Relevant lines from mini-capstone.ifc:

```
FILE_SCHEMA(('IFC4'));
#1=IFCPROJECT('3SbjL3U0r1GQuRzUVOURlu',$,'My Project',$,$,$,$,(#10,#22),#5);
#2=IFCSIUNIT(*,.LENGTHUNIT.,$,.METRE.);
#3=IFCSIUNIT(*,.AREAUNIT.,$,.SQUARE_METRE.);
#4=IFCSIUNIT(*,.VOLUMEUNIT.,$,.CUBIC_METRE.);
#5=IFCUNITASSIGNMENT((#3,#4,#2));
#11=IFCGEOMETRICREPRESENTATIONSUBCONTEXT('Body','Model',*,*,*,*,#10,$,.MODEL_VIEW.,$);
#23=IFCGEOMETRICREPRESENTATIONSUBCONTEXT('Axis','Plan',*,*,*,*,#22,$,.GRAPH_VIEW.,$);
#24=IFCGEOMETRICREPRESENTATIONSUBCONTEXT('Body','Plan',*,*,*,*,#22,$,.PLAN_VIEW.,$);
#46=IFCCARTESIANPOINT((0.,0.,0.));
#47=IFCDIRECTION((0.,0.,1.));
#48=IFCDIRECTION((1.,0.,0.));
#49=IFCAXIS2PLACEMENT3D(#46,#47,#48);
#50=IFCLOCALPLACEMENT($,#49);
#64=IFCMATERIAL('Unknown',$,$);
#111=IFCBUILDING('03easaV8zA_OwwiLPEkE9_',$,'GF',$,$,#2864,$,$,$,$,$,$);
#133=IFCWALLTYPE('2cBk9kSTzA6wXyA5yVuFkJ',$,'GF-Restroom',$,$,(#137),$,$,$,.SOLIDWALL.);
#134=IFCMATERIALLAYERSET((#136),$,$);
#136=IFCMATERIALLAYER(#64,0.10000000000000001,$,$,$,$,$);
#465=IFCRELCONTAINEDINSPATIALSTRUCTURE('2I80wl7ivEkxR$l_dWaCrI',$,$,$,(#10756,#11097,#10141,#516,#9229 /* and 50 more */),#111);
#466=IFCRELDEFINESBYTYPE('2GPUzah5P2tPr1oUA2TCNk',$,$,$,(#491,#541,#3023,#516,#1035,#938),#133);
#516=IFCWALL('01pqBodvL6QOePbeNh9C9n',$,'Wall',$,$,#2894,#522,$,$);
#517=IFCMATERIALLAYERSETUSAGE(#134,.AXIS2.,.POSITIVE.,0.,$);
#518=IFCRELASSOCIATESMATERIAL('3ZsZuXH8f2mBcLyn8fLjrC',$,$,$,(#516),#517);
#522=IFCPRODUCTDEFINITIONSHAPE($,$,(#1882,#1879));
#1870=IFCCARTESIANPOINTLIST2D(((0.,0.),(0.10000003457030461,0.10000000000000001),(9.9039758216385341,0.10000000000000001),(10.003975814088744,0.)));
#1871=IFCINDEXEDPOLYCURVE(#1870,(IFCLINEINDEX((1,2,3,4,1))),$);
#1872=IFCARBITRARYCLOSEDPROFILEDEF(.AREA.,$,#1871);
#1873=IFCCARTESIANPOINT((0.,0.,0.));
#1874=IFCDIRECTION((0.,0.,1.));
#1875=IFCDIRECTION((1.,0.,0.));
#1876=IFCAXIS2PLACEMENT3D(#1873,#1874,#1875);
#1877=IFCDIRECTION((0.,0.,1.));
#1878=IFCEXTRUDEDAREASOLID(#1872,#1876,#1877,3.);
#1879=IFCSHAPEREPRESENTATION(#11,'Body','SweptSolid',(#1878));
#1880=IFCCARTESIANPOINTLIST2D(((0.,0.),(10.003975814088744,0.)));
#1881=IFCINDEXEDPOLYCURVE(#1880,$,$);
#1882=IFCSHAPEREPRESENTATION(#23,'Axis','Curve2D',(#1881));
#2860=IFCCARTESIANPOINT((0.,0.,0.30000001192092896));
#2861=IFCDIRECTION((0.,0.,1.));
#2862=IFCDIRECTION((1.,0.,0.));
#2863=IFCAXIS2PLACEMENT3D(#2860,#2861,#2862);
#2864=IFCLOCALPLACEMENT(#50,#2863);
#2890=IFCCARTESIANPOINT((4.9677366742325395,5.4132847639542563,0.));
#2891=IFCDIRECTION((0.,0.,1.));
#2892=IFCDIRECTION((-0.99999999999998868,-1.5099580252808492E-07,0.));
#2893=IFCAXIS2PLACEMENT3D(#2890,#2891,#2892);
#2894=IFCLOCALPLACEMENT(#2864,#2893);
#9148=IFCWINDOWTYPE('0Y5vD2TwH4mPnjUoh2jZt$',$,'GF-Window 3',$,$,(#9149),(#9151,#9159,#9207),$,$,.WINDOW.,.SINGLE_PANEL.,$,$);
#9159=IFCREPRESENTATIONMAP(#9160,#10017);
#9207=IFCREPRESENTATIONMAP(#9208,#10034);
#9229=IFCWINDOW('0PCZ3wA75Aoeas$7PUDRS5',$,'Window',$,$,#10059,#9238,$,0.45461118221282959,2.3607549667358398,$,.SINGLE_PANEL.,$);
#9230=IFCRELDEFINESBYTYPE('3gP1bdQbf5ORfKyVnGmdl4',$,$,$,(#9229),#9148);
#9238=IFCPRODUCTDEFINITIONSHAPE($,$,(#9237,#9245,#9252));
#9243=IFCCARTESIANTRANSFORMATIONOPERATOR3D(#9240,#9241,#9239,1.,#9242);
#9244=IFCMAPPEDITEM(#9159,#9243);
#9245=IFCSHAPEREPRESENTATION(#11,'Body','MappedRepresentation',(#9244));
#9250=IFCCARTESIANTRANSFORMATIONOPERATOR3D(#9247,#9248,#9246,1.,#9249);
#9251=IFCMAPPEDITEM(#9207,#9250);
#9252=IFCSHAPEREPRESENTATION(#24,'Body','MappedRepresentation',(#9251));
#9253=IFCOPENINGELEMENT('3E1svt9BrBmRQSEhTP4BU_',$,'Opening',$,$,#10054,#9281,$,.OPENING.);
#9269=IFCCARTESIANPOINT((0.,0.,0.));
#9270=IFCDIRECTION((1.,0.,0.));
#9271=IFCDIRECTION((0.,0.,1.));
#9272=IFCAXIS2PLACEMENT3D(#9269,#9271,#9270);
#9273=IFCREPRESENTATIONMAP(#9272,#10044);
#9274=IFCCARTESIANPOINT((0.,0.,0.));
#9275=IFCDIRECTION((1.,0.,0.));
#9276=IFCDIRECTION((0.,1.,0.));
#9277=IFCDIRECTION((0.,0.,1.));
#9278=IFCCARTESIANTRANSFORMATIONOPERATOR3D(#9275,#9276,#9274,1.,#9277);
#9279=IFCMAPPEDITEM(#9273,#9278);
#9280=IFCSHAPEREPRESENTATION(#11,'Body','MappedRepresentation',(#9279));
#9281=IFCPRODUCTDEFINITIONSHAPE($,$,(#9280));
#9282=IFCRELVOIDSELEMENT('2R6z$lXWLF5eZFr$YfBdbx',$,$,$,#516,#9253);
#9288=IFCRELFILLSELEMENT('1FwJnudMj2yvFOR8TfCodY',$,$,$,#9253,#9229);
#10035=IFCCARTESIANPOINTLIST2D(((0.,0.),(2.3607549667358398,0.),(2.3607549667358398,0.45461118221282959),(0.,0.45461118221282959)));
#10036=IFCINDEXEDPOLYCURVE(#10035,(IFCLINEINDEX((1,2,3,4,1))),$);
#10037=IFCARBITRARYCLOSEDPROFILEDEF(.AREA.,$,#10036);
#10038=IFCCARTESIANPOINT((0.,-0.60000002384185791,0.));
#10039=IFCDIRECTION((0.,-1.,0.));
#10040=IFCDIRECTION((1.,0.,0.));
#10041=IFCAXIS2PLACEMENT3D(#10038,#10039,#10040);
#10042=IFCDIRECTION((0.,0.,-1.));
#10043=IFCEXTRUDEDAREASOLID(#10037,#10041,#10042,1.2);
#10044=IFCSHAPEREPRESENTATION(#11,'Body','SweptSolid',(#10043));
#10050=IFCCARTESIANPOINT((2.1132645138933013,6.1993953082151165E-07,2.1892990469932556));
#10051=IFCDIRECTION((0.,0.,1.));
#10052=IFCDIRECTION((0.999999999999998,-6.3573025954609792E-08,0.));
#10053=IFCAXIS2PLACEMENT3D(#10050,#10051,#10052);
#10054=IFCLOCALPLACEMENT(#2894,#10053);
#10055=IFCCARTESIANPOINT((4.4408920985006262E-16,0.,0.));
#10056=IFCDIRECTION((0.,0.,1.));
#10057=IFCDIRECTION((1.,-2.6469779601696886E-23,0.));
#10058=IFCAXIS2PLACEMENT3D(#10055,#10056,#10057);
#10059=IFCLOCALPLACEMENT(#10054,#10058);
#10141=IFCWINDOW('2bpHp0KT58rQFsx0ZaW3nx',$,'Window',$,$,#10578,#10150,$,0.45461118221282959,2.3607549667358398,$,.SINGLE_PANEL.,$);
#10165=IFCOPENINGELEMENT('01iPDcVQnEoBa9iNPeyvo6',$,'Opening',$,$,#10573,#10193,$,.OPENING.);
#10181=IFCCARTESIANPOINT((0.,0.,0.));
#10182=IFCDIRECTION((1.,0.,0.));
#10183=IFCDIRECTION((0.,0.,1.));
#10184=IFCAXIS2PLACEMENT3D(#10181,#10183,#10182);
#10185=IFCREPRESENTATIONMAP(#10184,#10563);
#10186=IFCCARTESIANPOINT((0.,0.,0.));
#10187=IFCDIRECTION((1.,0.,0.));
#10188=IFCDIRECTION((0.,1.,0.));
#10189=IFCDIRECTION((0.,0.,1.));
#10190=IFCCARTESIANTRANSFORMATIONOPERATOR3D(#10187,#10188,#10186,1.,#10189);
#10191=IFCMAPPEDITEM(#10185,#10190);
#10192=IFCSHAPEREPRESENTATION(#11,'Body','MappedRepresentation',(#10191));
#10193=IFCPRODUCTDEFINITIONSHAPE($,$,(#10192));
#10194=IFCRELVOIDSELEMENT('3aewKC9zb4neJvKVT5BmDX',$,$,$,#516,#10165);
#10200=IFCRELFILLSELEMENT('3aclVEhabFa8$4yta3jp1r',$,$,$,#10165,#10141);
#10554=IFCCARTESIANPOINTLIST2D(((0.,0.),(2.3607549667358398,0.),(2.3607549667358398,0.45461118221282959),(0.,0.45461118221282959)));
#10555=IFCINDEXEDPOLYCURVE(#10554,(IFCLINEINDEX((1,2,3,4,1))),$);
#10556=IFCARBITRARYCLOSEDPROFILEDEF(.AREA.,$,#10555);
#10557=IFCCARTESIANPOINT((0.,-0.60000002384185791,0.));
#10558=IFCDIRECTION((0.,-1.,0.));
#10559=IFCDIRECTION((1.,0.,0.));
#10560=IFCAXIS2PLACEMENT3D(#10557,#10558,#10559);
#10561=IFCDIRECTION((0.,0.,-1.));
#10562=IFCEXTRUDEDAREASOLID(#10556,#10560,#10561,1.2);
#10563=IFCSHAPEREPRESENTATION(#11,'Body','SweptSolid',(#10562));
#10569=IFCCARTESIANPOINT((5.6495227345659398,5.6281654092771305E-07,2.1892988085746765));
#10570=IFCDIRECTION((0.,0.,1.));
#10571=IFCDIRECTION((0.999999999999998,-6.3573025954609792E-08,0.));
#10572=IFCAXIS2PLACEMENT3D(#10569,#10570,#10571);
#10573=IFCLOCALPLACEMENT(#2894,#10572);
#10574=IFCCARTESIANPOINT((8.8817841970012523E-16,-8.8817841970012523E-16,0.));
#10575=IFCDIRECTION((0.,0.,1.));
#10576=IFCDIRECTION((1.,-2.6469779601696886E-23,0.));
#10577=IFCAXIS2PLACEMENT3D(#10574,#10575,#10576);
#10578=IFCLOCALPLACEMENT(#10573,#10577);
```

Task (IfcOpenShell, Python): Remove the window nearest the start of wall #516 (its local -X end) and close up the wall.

```python
import ifcopenshell
import ifcopenshell.api.feature
import ifcopenshell.api.root
import ifcopenshell.geom
import ifcopenshell.util.shape

model = ifcopenshell.open("mini-capstone.ifc")
settings = ifcopenshell.geom.settings()


def volume(element):
    """Net volume in cubic metres, openings subtracted."""
    shape = ifcopenshell.geom.create_shape(settings, element)
    return ifcopenshell.util.shape.get_volume(shape.geometry)


window = model.by_guid("0PCZ3wA75Aoeas$7PUDRS5")
opening = window.FillsVoids[0].RelatingOpeningElement
wall = opening.VoidsElements[0].RelatingBuildingElement
before = volume(wall)

ifcopenshell.api.root.remove_product(model, product=window)
ifcopenshell.api.feature.remove_feature(model, feature=opening)

after = volume(wall)

print(f"wall volume {before:.3f} -> {after:.3f} m3")

model.write("mini-capstone-out.ifc")
```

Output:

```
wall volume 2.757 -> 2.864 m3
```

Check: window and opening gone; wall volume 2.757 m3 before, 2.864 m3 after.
